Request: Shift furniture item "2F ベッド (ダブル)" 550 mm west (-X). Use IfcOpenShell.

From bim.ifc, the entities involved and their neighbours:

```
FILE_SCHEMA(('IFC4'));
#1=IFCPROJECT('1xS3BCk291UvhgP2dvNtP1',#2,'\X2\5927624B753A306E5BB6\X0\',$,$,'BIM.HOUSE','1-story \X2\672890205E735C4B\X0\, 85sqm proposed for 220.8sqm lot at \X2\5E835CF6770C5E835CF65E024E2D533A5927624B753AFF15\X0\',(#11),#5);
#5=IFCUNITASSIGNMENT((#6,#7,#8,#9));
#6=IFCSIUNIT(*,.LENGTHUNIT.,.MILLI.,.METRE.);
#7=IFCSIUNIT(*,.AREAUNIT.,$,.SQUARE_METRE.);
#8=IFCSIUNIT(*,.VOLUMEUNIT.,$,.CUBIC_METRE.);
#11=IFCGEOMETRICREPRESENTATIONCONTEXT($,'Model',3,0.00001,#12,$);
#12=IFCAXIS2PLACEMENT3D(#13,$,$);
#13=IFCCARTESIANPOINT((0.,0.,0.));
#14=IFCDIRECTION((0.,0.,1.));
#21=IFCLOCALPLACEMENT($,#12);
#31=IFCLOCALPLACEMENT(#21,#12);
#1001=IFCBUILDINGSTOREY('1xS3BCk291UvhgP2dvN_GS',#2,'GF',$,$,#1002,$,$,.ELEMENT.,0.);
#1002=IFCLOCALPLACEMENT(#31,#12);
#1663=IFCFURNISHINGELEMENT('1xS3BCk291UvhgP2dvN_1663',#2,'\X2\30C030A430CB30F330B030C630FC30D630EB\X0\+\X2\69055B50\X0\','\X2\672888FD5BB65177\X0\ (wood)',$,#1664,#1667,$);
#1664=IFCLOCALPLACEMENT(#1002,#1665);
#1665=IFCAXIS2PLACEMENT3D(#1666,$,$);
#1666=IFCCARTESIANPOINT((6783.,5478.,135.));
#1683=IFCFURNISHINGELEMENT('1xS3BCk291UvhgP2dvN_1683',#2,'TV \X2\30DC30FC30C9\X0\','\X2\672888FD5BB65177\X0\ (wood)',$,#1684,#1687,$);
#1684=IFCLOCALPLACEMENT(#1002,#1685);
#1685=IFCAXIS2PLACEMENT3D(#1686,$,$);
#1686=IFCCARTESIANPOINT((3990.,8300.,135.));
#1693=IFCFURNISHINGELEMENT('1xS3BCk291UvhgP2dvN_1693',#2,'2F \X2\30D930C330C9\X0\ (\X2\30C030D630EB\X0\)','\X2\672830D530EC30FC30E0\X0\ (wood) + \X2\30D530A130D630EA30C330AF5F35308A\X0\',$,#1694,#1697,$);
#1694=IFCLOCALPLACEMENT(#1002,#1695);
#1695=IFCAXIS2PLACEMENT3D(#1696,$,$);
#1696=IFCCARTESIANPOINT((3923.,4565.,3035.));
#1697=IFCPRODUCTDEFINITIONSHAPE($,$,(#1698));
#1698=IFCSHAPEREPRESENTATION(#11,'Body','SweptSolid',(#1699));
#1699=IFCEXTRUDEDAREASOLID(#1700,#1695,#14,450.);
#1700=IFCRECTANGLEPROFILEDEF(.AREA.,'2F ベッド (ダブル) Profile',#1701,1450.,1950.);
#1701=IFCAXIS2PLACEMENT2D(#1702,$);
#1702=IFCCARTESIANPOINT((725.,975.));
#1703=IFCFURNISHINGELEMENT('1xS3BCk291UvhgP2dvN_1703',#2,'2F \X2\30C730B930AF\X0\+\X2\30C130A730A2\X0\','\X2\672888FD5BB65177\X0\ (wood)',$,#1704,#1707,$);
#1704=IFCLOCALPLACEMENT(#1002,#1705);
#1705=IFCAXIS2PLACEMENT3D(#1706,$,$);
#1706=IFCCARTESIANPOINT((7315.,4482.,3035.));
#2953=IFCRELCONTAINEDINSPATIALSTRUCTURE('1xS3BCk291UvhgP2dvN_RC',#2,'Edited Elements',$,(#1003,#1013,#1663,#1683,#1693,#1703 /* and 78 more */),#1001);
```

```python
import ifcopenshell
import ifcopenshell.api.geometry
import ifcopenshell.util.placement

model = ifcopenshell.open("bim.ifc")

item = model.by_guid("1xS3BCk291UvhgP2dvN_1693")
matrix = ifcopenshell.util.placement.get_local_placement(item.ObjectPlacement)
matrix[0, 3] -= 550.0
ifcopenshell.api.geometry.edit_object_placement(model, product=item, matrix=matrix, is_si=False)

print(ifcopenshell.util.placement.get_local_placement(item.ObjectPlacement).round(3) + 0.0)

model.write("bim-out.ifc")
```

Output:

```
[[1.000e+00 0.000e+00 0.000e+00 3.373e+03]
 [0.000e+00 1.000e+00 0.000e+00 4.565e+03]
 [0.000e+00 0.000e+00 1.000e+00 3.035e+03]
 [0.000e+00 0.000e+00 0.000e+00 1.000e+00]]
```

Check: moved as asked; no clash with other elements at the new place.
